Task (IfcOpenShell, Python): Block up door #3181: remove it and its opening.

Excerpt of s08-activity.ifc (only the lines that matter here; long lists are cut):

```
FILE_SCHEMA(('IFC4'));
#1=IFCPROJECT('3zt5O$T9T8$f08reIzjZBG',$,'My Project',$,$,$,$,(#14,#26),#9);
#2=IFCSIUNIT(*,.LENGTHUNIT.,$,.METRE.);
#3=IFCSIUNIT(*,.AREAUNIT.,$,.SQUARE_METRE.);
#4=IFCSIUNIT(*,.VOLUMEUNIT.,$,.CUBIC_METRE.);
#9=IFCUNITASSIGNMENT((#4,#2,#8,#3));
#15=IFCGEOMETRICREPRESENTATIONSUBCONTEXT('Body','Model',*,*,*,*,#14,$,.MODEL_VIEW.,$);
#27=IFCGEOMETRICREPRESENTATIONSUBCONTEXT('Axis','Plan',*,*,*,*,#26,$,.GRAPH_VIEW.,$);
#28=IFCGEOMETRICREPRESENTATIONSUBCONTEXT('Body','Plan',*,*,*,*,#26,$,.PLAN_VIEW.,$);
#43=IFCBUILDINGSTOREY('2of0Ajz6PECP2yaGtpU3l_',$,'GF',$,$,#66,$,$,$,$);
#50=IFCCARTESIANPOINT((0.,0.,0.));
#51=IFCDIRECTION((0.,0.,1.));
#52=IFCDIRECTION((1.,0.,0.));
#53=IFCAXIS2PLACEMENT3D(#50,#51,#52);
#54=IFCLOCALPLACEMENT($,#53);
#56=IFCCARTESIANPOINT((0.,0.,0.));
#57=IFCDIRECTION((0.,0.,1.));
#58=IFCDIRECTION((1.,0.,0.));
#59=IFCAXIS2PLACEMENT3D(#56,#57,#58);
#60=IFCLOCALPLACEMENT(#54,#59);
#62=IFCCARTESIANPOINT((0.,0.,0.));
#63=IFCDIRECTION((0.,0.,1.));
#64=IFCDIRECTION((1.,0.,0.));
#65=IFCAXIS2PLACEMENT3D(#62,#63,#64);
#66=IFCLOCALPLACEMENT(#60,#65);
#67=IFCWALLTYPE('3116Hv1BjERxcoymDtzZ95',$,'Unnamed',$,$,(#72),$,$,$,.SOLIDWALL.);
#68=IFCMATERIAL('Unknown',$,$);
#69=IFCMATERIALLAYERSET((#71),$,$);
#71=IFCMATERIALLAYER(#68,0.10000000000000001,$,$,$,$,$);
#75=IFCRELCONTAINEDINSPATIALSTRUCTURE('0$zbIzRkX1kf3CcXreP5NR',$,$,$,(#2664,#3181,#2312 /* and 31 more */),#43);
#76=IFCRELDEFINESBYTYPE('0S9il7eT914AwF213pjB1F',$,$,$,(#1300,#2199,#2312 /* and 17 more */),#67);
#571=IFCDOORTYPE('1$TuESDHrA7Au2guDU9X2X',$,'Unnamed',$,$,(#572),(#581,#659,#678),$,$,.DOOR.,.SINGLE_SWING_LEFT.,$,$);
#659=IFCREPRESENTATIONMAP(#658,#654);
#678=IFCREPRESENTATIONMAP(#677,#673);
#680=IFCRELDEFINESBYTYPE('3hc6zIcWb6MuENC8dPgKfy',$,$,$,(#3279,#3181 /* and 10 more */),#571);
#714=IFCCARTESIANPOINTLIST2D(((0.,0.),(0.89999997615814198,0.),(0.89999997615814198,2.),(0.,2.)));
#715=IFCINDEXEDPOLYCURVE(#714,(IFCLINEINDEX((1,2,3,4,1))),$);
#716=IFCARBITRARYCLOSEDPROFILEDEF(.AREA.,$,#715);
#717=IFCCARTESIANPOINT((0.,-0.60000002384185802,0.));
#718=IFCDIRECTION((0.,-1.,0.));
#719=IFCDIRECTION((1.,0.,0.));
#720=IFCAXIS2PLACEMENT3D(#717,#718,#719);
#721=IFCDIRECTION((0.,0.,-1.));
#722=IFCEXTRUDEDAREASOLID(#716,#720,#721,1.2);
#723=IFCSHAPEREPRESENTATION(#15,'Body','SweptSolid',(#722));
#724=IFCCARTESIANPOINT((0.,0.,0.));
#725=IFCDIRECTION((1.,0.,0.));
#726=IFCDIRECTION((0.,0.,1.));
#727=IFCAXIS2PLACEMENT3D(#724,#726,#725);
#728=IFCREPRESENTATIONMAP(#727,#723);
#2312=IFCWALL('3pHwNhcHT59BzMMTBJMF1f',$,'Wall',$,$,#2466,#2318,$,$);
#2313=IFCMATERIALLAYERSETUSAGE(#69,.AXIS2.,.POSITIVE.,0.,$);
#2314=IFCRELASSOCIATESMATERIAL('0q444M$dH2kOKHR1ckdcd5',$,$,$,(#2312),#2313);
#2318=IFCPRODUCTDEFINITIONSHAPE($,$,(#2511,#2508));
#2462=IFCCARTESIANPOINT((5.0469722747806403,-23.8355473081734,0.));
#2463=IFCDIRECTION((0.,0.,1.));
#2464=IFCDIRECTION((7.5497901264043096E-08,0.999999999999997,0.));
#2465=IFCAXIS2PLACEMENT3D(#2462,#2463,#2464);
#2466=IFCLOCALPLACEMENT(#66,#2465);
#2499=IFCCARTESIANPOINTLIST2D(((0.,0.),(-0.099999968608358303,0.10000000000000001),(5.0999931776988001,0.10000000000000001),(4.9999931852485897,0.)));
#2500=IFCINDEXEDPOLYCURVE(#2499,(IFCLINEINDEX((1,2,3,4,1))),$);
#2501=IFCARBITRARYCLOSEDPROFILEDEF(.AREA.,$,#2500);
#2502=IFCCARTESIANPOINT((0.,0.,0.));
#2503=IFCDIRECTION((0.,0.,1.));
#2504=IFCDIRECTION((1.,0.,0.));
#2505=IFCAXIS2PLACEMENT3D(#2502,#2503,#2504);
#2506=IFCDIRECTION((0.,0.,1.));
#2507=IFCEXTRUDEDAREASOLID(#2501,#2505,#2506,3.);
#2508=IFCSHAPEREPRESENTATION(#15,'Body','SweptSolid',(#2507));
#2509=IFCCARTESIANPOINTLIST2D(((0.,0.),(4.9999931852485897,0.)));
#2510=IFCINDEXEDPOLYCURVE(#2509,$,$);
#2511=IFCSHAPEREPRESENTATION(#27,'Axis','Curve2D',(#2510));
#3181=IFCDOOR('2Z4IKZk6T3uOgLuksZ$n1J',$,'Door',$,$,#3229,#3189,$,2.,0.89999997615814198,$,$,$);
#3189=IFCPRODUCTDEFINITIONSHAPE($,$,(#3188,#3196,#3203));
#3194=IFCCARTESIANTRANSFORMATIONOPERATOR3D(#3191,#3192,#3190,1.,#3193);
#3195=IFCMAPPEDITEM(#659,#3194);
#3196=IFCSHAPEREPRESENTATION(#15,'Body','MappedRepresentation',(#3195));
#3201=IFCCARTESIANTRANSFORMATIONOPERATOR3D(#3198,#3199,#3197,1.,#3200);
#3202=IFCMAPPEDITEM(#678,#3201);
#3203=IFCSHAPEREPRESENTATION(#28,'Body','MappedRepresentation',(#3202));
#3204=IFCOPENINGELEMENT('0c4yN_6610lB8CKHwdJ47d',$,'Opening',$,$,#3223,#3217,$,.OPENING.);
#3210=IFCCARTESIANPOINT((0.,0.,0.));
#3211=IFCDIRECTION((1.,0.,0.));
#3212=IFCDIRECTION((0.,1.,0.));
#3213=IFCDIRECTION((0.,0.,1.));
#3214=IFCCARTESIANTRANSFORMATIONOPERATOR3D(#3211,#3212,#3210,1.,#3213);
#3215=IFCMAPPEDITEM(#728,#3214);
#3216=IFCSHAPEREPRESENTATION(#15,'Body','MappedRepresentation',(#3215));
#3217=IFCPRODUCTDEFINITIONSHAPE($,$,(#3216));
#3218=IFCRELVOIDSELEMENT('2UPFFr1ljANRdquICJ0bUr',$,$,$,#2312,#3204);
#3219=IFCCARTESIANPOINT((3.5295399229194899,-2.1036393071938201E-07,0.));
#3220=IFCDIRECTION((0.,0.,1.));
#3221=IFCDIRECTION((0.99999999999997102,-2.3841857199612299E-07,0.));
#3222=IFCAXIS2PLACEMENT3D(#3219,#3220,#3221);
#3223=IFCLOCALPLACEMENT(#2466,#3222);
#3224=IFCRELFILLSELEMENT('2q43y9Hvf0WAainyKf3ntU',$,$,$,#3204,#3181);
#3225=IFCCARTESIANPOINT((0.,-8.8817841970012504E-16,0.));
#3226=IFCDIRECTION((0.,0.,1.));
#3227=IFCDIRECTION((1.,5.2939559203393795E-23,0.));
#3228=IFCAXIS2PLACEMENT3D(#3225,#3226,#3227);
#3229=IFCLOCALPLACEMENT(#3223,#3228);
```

```python
import ifcopenshell
import ifcopenshell.api.feature
import ifcopenshell.api.root
import ifcopenshell.geom
import ifcopenshell.util.shape

model = ifcopenshell.open("s08-activity.ifc")
settings = ifcopenshell.geom.settings()


def volume(element):
    """Net volume in cubic metres, openings subtracted."""
    shape = ifcopenshell.geom.create_shape(settings, element)
    return ifcopenshell.util.shape.get_volume(shape.geometry)


door = model.by_id(3181)
opening = door.FillsVoids[0].RelatingOpeningElement
wall = opening.VoidsElements[0].RelatingBuildingElement
before = volume(wall)

ifcopenshell.api.root.remove_product(model, product=door)
ifcopenshell.api.feature.remove_feature(model, feature=opening)

after = volume(wall)

print(f"wall volume {before:.3f} -> {after:.3f} m3")

model.write("s08-activity_edited.ifc")
```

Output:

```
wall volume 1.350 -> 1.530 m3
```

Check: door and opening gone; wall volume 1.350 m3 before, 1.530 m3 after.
